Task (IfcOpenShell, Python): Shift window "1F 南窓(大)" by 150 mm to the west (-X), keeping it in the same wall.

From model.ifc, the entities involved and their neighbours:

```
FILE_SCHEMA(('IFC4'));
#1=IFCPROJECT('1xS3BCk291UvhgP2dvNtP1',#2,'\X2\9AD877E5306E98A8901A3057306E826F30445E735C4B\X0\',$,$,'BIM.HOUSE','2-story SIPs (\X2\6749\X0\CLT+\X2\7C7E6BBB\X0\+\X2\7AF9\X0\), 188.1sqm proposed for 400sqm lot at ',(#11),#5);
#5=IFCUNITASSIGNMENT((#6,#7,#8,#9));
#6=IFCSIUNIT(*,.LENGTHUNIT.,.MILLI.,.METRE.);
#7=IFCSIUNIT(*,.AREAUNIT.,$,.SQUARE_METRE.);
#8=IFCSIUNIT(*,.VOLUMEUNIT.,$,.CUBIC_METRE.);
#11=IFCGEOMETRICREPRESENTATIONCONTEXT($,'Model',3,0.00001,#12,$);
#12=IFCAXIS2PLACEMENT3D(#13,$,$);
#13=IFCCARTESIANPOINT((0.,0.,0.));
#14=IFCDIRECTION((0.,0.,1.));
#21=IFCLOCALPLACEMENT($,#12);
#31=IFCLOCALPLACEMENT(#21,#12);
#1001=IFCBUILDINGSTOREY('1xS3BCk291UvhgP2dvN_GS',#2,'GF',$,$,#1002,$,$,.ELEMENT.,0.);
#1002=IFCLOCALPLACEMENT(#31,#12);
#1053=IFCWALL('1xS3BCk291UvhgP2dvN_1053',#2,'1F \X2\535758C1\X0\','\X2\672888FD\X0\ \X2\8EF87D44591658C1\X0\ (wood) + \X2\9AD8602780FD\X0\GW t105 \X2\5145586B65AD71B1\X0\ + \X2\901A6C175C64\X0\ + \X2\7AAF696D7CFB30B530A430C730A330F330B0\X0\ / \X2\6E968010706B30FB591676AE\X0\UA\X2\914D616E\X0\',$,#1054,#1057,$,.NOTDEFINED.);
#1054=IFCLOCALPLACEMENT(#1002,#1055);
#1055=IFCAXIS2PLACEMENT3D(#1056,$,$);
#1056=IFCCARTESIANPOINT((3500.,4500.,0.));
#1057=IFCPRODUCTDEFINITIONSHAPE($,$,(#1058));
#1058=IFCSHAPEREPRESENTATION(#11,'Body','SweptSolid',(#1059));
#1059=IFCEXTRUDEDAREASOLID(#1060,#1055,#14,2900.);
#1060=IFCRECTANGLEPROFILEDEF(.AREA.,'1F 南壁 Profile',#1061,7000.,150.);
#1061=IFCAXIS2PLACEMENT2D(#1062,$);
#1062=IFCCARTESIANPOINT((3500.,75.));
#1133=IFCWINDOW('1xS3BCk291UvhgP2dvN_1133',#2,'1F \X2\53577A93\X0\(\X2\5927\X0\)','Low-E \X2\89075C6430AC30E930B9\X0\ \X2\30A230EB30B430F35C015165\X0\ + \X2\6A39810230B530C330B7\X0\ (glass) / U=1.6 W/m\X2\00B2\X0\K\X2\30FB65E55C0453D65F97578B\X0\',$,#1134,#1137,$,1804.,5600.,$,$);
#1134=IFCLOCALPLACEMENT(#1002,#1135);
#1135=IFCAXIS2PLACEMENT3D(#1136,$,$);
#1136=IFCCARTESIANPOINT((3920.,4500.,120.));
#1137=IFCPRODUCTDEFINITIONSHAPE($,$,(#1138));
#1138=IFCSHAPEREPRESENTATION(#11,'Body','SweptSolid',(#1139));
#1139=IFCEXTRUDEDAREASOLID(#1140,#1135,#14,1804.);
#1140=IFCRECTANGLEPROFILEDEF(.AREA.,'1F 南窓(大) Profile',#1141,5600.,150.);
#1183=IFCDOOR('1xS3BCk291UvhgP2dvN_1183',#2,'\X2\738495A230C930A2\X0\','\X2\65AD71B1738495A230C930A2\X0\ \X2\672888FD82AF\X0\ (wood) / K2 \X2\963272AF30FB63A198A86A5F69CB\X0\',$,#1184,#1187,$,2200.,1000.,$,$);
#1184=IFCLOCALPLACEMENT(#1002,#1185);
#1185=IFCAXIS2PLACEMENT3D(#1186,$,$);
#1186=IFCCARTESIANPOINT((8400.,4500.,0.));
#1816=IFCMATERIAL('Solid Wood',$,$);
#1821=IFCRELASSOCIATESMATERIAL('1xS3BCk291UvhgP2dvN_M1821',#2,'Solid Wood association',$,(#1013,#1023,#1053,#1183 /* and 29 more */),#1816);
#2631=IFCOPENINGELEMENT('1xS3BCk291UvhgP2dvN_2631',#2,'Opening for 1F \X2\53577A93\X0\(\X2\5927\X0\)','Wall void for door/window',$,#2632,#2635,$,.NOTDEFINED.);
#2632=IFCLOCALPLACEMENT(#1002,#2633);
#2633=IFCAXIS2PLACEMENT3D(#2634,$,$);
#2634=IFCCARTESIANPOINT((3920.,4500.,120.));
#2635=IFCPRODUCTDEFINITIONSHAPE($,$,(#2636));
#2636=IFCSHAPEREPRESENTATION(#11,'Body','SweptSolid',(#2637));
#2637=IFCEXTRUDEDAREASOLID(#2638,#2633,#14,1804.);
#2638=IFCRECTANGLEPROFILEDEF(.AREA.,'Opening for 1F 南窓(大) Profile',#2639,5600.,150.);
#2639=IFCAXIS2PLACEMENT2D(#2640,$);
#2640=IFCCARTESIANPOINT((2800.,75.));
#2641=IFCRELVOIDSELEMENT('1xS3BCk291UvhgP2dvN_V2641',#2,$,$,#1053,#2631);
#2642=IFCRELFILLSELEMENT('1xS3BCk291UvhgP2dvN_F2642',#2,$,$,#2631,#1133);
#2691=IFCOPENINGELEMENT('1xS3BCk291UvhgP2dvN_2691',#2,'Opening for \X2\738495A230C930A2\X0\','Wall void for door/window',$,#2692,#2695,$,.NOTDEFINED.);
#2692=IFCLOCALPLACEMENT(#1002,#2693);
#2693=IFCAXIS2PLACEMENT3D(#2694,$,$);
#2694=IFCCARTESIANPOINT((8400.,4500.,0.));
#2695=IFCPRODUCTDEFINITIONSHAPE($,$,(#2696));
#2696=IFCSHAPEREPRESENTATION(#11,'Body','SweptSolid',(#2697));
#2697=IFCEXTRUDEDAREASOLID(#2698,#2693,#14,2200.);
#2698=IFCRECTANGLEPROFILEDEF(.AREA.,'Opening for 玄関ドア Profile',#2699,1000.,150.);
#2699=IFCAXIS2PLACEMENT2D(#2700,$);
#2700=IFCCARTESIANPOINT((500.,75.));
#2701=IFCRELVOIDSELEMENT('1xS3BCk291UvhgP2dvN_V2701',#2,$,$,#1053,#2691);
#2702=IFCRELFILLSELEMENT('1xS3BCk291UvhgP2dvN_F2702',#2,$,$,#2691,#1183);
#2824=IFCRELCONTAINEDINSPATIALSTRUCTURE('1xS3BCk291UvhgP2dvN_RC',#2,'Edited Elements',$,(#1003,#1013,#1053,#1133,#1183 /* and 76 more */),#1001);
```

```python
import ifcopenshell
import ifcopenshell.api.geometry
import ifcopenshell.util.placement

model = ifcopenshell.open("model.ifc")

window = model.by_guid("1xS3BCk291UvhgP2dvN_1133")
opening = window.FillsVoids[0].RelatingOpeningElement
wall = opening.VoidsElements[0].RelatingBuildingElement

wall_matrix = ifcopenshell.util.placement.get_local_placement(wall.ObjectPlacement)
shift = wall_matrix[:3, 0] * -150.0
before = ifcopenshell.util.placement.get_local_placement(window.ObjectPlacement)[:3, 3].copy()

# The window is not placed relative to its opening, so move both.
for product in (opening, window):
    matrix = ifcopenshell.util.placement.get_local_placement(product.ObjectPlacement)
    matrix[:3, 3] += shift
    ifcopenshell.api.geometry.edit_object_placement(model, product=product, matrix=matrix, is_si=False)

after = ifcopenshell.util.placement.get_local_placement(window.ObjectPlacement)[:3, 3]
print("window moved by", (after - before).round(3) + 0.0)

model.write("model_rev.ifc")
```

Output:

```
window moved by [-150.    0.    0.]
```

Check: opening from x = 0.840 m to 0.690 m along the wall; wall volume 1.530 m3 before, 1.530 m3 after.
